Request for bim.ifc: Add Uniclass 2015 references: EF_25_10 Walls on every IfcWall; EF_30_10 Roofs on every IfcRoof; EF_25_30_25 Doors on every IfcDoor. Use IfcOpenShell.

First a look at what the model holds.

```python
import ifcopenshell

model = ifcopenshell.open("bim.ifc")
print(model.schema)
print("classifications:", [c.Name for c in model.by_type("IfcClassification")])
for ifc_class in ("IfcDoor", "IfcRoof", "IfcStair", "IfcWall", "IfcWindow"):
    print(ifc_class, len(model.by_type(ifc_class)))
```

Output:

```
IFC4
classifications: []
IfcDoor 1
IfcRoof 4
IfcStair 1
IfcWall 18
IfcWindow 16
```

```python
import ifcopenshell
import ifcopenshell.api.classification

model = ifcopenshell.open("bim.ifc")

system = ifcopenshell.api.classification.add_classification(model, classification="Uniclass 2015")

codes = {
    "IfcWall": ("EF_25_10", "Walls"),
    "IfcRoof": ("EF_30_10", "Roofs"),
    "IfcDoor": ("EF_25_30_25", "Doors"),
}
for ifc_class, (code, name) in codes.items():
    products = model.by_type(ifc_class)
    ifcopenshell.api.classification.add_reference(
        model, products=products, classification=system, identification=code, name=name
    )
    print(code, len(products))

model.write("bim_edited.ifc")
```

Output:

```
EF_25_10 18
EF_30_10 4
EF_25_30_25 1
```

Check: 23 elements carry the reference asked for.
